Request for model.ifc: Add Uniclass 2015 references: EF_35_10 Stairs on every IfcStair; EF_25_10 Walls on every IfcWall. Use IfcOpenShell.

First a look at what the model holds.

```python
import ifcopenshell

model = ifcopenshell.open("model.ifc")
print(model.schema)
print("classifications:", [c.Name for c in model.by_type("IfcClassification")])
for ifc_class in ("IfcDoor", "IfcRoof", "IfcStair", "IfcWall", "IfcWindow"):
    print(ifc_class, len(model.by_type(ifc_class)))
```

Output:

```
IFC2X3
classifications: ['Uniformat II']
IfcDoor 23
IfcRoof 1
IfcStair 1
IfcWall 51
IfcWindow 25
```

```python
import ifcopenshell
import ifcopenshell.api.classification

model = ifcopenshell.open("model.ifc")

# IFC2X3 requires Source and Edition and has no link from the project to the system.
system = model.create_entity("IfcClassification", Source="NBS", Edition="2015", Name="Uniclass 2015")

codes = {
    "IfcStair": ("EF_35_10", "Stairs"),
    "IfcWall": ("EF_25_10", "Walls"),
}
for ifc_class, (code, name) in codes.items():
    products = model.by_type(ifc_class)
    ifcopenshell.api.classification.add_reference(
        model, products=products, classification=system, identification=code, name=name
    )
    print(code, len(products))

model.write("model_v2.ifc")
```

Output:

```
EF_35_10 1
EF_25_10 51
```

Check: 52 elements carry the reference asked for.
